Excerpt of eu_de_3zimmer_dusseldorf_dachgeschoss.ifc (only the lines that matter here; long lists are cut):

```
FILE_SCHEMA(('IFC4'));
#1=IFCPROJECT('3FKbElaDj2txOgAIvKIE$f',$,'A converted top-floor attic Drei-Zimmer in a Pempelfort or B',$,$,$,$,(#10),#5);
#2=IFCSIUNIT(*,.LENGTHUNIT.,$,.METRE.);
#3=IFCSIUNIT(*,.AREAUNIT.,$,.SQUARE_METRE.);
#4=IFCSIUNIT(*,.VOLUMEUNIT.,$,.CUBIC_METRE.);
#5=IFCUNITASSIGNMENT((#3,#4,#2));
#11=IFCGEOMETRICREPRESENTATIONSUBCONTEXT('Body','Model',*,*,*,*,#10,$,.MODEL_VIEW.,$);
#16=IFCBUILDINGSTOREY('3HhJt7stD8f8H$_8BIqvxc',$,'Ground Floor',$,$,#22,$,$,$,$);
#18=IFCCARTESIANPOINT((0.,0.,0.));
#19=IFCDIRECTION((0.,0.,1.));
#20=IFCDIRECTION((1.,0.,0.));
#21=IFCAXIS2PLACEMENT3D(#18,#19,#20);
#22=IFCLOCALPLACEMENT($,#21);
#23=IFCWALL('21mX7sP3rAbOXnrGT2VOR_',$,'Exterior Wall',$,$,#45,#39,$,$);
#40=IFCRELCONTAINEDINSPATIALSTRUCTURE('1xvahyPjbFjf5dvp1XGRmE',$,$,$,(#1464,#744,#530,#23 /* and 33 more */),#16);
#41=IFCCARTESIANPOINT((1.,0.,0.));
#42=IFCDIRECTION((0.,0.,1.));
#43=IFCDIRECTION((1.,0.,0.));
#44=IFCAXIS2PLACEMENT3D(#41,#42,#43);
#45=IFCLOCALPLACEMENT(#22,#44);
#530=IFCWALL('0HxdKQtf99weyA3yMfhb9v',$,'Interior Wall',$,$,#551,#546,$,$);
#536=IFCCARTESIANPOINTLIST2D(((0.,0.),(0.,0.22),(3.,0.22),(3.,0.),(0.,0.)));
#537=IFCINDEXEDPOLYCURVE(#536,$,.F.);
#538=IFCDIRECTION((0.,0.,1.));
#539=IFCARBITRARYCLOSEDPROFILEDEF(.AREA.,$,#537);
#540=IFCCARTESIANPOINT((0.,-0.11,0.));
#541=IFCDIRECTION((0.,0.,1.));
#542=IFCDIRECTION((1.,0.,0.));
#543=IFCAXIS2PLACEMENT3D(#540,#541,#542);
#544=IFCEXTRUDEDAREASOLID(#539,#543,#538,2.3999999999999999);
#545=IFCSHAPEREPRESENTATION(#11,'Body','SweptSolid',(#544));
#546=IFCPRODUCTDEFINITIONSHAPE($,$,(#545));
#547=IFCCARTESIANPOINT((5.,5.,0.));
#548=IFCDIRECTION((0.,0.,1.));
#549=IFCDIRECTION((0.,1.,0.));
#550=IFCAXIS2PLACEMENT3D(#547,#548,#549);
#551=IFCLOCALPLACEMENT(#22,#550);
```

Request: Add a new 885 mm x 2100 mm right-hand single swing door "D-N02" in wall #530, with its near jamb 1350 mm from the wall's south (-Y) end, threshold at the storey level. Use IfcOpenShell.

```python
import numpy as np
import ifcopenshell
import ifcopenshell.api.feature
import ifcopenshell.api.geometry
import ifcopenshell.api.root
import ifcopenshell.api.spatial
import ifcopenshell.geom
import ifcopenshell.util.element
import ifcopenshell.util.placement
import ifcopenshell.util.representation
import ifcopenshell.util.shape
import ifcopenshell.util.unit

model = ifcopenshell.open("eu_de_3zimmer_dusseldorf_dachgeschoss.ifc")
unit_scale = ifcopenshell.util.unit.calculate_unit_scale(model)
settings = ifcopenshell.geom.settings()


def volume(element):
    """Net volume in cubic metres, openings subtracted."""
    shape = ifcopenshell.geom.create_shape(settings, element)
    return ifcopenshell.util.shape.get_volume(shape.geometry)


wall = model.by_guid("0HxdKQtf99weyA3yMfhb9v")
storey = ifcopenshell.util.element.get_container(wall, ifc_class="IfcBuildingStorey")
context = ifcopenshell.util.representation.get_context(model, "Model", "Body", "MODEL_VIEW")
before = volume(wall)

width, height, from_end, sill = 0.885, 2.1, 1.35, 0.0  # metres

# The wall runs along its own X axis, and the end named is its -X end.
wall_shape = ifcopenshell.geom.create_shape(settings, wall)
x, y, z = ifcopenshell.util.shape.get_vertices(wall_shape.geometry).T
start = x.min() + from_end
face, thickness = float(y.min()), float(y.max() - y.min())
wall_matrix = ifcopenshell.util.placement.get_local_placement(wall.ObjectPlacement)
level = ifcopenshell.util.placement.get_local_placement(storey.ObjectPlacement)[2, 3]


def in_wall(x, y):
    """Placement at x, y metres in the wall's axes, at sill height."""
    matrix = wall_matrix.copy()
    matrix[:, 3] = wall_matrix @ np.array([x / unit_scale, y / unit_scale, 0.0, 1.0])
    matrix[2, 3] = level + sill / unit_scale
    return matrix


# Opening: a box that overshoots both wall faces by 50 mm.
opening = ifcopenshell.api.root.create_entity(model, ifc_class="IfcOpeningElement", predefined_type="OPENING")
box = ifcopenshell.api.geometry.add_wall_representation(
    model, context=context, length=width, height=height, thickness=thickness + 0.1
)
ifcopenshell.api.geometry.assign_representation(model, product=opening, representation=box)
ifcopenshell.api.geometry.edit_object_placement(model, product=opening, matrix=in_wall(start, face - 0.05), is_si=False)
ifcopenshell.api.feature.add_feature(model, feature=opening, element=wall)

door = ifcopenshell.api.root.create_entity(model, ifc_class="IfcDoor", name="D-N02", predefined_type="DOOR")
door.OverallWidth, door.OverallHeight = width / unit_scale, height / unit_scale
door.OperationType = "SINGLE_SWING_RIGHT"
body = ifcopenshell.api.geometry.add_door_representation(
    model,
    context=context,
    overall_width=door.OverallWidth,
    overall_height=door.OverallHeight,
    operation_type="SINGLE_SWING_RIGHT",
    lining_properties={"LiningDepth": thickness / unit_scale, "ThresholdDepth": thickness / unit_scale},
)
ifcopenshell.api.geometry.assign_representation(model, product=door, representation=body)
ifcopenshell.api.spatial.assign_container(model, products=[door], relating_structure=storey)
ifcopenshell.api.feature.add_filling(model, opening=opening, element=door)

# The lining spans the wall, so the door starts at the wall face.
ifcopenshell.api.geometry.edit_object_placement(model, product=door, matrix=in_wall(start, face), is_si=False)

after = volume(wall)

print(f"wall volume {before:.3f} -> {after:.3f} m3")

model.write("eu_de_3zimmer_dusseldorf_dachgeschoss_rev.ifc")
```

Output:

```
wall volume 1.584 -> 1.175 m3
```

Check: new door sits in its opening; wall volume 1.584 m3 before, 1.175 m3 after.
